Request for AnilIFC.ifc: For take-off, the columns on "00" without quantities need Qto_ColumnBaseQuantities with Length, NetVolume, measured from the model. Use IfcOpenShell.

First a look at what the model holds.

```python
import ifcopenshell
import ifcopenshell.util.element
import ifcopenshell.util.unit

model = ifcopenshell.open("AnilIFC.ifc")
print(model.schema)
for unit_type in ("LENGTHUNIT", "AREAUNIT", "VOLUMEUNIT"):
    print(unit_type, ifcopenshell.util.unit.calculate_unit_scale(model, unit_type))
storey = next(s for s in model.by_type("IfcBuildingStorey") if s.Name == "00")
columns = [e for e in ifcopenshell.util.element.get_decomposition(storey) if e.is_a("IfcColumn")]
for e in sorted(columns, key=lambda e: e.id()):
    print(e.id(), e.is_a(), e.Name, list(ifcopenshell.util.element.get_psets(e, qtos_only=True)), sep=" | ")
```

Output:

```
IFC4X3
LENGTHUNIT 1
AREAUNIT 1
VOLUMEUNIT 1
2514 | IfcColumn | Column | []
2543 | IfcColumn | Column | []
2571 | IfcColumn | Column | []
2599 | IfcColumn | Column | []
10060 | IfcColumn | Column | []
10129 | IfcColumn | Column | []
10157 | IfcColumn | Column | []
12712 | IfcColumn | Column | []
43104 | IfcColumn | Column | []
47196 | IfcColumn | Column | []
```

```python
import ifcopenshell
import ifcopenshell.api.pset
import ifcopenshell.geom
import ifcopenshell.util.element
import ifcopenshell.util.shape
import ifcopenshell.util.unit

model = ifcopenshell.open("AnilIFC.ifc")
unit_scale = ifcopenshell.util.unit.calculate_unit_scale(model)
volume_scale = ifcopenshell.util.unit.calculate_unit_scale(model, "VOLUMEUNIT")
settings = ifcopenshell.geom.settings()

storey = next(s for s in model.by_type("IfcBuildingStorey") if s.Name == "00")
columns = [e for e in ifcopenshell.util.element.get_decomposition(storey) if e.is_a("IfcColumn")]

for e in sorted(columns, key=lambda e: e.id()):
    if ifcopenshell.util.element.get_psets(e, qtos_only=True, should_inherit=False):
        continue
    # Geometry comes back in metres, in the element's own axes.
    shape = ifcopenshell.geom.create_shape(settings, e)
    values = {
        "Length": ifcopenshell.util.shape.get_z(shape.geometry) / unit_scale,
        "NetVolume": ifcopenshell.util.shape.get_volume(shape.geometry) / volume_scale,
    }
    qto = ifcopenshell.api.pset.add_qto(model, product=e, name="Qto_ColumnBaseQuantities")
    ifcopenshell.api.pset.edit_qto(model, qto=qto, properties=values)
    print(e.id(), {k: round(v, 3) for k, v in values.items()})

model.write("AnilIFC_rev.ifc")
```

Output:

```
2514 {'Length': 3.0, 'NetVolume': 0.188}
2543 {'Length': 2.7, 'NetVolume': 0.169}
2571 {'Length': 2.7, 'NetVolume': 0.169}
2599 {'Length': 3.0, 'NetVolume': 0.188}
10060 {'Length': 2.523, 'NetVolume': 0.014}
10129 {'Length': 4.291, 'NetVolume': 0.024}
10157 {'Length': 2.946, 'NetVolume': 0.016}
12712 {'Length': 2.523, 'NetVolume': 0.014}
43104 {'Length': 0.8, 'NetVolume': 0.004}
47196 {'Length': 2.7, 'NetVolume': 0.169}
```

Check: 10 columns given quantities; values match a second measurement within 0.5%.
